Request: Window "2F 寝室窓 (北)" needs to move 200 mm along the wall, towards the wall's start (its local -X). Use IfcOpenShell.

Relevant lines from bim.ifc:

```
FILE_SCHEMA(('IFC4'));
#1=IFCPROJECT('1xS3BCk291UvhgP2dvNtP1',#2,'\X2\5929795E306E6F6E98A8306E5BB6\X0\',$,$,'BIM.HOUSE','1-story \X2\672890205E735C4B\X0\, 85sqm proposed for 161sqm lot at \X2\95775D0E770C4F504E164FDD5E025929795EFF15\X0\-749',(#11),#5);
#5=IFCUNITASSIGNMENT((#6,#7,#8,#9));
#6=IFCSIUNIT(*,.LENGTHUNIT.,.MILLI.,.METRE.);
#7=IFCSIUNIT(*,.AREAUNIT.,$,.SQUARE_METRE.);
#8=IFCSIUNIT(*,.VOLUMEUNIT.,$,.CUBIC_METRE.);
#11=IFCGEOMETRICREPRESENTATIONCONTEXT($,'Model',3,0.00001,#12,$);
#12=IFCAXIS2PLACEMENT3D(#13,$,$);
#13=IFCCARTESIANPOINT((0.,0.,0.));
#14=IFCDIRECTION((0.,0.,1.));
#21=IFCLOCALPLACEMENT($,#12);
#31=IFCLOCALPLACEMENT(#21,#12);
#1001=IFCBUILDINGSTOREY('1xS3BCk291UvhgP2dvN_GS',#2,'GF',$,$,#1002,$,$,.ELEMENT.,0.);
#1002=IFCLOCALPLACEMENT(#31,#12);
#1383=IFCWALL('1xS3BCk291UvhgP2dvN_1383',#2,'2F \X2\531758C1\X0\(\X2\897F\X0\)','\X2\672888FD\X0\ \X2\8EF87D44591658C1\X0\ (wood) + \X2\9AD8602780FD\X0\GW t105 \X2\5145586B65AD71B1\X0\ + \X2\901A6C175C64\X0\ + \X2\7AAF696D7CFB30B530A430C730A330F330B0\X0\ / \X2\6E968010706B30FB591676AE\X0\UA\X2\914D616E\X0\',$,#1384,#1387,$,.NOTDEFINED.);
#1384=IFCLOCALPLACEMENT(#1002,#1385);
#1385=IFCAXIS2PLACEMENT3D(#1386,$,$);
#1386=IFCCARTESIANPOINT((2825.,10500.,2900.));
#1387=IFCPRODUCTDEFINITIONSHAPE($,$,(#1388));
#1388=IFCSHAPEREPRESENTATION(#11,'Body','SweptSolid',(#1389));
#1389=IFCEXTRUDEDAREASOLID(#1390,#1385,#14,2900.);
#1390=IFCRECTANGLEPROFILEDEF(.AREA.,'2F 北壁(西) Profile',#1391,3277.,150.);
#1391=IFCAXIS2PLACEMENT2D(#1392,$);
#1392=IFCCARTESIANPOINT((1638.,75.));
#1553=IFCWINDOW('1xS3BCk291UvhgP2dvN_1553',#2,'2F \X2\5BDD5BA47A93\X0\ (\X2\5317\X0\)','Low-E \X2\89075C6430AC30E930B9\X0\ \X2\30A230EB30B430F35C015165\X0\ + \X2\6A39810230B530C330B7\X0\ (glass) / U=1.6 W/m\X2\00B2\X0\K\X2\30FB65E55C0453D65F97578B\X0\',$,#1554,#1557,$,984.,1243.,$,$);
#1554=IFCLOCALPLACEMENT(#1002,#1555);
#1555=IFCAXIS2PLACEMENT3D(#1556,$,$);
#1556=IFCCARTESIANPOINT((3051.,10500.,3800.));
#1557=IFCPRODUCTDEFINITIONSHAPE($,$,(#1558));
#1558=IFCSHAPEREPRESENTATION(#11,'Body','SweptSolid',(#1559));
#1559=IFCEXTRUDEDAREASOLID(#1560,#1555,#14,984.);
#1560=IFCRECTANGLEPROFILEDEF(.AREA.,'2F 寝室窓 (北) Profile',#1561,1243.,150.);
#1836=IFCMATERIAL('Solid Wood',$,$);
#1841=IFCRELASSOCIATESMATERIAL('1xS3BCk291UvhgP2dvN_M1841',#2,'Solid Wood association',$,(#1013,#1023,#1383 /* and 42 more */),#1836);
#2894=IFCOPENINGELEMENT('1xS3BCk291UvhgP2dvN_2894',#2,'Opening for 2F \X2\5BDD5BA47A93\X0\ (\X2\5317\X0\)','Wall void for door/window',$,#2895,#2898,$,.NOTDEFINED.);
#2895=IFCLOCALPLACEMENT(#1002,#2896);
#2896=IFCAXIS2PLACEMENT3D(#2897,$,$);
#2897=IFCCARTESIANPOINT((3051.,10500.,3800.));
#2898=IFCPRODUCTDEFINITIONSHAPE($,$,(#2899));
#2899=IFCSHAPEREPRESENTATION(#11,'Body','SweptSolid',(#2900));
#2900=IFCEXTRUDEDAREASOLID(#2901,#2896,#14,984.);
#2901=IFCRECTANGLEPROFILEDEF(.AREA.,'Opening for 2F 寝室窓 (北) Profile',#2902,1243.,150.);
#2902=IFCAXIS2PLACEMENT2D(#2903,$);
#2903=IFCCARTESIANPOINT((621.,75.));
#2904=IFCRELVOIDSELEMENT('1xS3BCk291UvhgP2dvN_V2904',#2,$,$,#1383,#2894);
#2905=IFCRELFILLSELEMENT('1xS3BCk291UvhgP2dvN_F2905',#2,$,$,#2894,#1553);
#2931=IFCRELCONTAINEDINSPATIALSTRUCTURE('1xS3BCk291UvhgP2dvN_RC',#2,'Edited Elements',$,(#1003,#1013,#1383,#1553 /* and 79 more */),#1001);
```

```python
import ifcopenshell
import ifcopenshell.api.geometry
import ifcopenshell.util.placement

model = ifcopenshell.open("bim.ifc")

window = model.by_guid("1xS3BCk291UvhgP2dvN_1553")
opening = window.FillsVoids[0].RelatingOpeningElement
wall = opening.VoidsElements[0].RelatingBuildingElement

wall_matrix = ifcopenshell.util.placement.get_local_placement(wall.ObjectPlacement)
shift = wall_matrix[:3, 0] * -200.0
before = ifcopenshell.util.placement.get_local_placement(window.ObjectPlacement)[:3, 3].copy()

# The window is not placed relative to its opening, so move both.
for product in (opening, window):
    matrix = ifcopenshell.util.placement.get_local_placement(product.ObjectPlacement)
    matrix[:3, 3] += shift
    ifcopenshell.api.geometry.edit_object_placement(model, product=product, matrix=matrix, is_si=False)

after = ifcopenshell.util.placement.get_local_placement(window.ObjectPlacement)[:3, 3]
print("window moved by", (after - before).round(3) + 0.0)

model.write("bim_updated.ifc")
```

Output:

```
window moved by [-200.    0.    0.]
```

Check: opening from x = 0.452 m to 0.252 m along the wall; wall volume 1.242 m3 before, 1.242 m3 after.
